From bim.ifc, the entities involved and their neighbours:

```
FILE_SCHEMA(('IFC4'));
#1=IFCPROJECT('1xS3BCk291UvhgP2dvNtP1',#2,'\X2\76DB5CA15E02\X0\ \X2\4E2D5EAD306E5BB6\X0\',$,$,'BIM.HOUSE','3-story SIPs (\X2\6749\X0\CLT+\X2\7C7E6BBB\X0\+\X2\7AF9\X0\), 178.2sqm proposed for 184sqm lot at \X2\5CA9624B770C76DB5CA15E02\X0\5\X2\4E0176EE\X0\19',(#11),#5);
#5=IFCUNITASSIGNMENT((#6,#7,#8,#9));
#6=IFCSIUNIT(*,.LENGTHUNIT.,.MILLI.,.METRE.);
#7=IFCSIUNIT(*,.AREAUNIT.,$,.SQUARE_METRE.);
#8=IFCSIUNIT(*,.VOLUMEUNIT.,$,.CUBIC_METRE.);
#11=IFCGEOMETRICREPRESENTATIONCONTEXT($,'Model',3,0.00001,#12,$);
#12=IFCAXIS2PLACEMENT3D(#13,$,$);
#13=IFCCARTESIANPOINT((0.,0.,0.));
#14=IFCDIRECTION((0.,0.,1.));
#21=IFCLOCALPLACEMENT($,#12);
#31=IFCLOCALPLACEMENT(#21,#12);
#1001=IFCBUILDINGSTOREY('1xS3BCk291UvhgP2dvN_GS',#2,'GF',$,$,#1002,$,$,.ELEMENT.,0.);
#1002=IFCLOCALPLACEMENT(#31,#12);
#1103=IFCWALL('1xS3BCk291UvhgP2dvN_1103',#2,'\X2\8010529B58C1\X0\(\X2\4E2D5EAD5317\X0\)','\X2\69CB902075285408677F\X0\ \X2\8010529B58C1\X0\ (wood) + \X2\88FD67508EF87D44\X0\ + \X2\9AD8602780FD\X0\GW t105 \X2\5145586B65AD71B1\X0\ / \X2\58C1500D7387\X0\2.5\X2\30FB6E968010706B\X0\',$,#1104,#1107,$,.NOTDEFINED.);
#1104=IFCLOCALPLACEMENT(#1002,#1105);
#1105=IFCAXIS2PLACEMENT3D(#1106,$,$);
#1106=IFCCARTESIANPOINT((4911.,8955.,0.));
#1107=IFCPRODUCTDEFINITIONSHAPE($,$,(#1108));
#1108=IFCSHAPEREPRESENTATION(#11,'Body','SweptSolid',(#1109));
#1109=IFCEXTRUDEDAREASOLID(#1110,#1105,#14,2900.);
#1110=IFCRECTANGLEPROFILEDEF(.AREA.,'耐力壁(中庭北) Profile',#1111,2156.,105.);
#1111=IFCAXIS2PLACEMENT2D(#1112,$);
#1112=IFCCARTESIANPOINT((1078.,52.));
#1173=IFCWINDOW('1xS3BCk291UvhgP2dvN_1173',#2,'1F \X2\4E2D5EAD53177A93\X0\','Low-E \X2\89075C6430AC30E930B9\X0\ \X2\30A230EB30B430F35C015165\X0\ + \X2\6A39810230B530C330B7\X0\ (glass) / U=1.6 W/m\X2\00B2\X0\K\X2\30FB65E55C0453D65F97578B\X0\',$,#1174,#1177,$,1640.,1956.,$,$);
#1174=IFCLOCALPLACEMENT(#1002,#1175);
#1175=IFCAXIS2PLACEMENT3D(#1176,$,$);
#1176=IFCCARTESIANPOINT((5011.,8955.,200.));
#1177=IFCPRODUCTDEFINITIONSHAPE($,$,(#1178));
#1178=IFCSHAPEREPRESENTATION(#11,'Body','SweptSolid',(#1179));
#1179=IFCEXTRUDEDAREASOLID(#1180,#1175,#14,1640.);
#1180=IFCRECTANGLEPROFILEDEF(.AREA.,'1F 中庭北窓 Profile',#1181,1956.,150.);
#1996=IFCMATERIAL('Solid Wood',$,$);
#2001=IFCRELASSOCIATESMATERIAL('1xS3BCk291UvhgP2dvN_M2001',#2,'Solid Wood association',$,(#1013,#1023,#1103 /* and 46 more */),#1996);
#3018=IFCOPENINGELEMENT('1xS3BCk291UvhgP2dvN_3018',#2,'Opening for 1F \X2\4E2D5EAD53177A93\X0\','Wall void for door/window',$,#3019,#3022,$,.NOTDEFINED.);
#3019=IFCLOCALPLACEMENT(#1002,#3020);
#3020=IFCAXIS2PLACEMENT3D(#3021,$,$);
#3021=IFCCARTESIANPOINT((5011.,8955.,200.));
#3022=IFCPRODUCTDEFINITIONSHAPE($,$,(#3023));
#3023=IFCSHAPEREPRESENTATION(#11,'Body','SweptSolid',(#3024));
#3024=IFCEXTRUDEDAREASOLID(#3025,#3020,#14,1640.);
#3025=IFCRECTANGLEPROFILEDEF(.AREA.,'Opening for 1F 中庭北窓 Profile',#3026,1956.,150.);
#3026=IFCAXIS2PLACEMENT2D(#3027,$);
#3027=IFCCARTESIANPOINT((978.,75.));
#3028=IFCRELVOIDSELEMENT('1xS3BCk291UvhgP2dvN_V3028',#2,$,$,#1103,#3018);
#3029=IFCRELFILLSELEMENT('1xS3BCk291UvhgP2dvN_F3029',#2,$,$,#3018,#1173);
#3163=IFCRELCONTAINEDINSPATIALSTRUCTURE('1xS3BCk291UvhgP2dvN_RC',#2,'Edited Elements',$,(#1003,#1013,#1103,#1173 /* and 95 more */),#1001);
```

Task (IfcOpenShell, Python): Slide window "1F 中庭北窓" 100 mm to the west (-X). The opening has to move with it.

```python
import ifcopenshell
import ifcopenshell.api.geometry
import ifcopenshell.util.placement

model = ifcopenshell.open("bim.ifc")

window = model.by_guid("1xS3BCk291UvhgP2dvN_1173")
opening = window.FillsVoids[0].RelatingOpeningElement
wall = opening.VoidsElements[0].RelatingBuildingElement

wall_matrix = ifcopenshell.util.placement.get_local_placement(wall.ObjectPlacement)
shift = wall_matrix[:3, 0] * -100.0
before = ifcopenshell.util.placement.get_local_placement(window.ObjectPlacement)[:3, 3].copy()

# The window is not placed relative to its opening, so move both.
for product in (opening, window):
    matrix = ifcopenshell.util.placement.get_local_placement(product.ObjectPlacement)
    matrix[:3, 3] += shift
    ifcopenshell.api.geometry.edit_object_placement(model, product=product, matrix=matrix, is_si=False)

after = ifcopenshell.util.placement.get_local_placement(window.ObjectPlacement)[:3, 3]
print("window moved by", (after - before).round(3) + 0.0)

model.write("bim_v2.ifc")
```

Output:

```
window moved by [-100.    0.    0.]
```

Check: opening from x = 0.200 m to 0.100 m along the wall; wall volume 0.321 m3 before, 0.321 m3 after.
